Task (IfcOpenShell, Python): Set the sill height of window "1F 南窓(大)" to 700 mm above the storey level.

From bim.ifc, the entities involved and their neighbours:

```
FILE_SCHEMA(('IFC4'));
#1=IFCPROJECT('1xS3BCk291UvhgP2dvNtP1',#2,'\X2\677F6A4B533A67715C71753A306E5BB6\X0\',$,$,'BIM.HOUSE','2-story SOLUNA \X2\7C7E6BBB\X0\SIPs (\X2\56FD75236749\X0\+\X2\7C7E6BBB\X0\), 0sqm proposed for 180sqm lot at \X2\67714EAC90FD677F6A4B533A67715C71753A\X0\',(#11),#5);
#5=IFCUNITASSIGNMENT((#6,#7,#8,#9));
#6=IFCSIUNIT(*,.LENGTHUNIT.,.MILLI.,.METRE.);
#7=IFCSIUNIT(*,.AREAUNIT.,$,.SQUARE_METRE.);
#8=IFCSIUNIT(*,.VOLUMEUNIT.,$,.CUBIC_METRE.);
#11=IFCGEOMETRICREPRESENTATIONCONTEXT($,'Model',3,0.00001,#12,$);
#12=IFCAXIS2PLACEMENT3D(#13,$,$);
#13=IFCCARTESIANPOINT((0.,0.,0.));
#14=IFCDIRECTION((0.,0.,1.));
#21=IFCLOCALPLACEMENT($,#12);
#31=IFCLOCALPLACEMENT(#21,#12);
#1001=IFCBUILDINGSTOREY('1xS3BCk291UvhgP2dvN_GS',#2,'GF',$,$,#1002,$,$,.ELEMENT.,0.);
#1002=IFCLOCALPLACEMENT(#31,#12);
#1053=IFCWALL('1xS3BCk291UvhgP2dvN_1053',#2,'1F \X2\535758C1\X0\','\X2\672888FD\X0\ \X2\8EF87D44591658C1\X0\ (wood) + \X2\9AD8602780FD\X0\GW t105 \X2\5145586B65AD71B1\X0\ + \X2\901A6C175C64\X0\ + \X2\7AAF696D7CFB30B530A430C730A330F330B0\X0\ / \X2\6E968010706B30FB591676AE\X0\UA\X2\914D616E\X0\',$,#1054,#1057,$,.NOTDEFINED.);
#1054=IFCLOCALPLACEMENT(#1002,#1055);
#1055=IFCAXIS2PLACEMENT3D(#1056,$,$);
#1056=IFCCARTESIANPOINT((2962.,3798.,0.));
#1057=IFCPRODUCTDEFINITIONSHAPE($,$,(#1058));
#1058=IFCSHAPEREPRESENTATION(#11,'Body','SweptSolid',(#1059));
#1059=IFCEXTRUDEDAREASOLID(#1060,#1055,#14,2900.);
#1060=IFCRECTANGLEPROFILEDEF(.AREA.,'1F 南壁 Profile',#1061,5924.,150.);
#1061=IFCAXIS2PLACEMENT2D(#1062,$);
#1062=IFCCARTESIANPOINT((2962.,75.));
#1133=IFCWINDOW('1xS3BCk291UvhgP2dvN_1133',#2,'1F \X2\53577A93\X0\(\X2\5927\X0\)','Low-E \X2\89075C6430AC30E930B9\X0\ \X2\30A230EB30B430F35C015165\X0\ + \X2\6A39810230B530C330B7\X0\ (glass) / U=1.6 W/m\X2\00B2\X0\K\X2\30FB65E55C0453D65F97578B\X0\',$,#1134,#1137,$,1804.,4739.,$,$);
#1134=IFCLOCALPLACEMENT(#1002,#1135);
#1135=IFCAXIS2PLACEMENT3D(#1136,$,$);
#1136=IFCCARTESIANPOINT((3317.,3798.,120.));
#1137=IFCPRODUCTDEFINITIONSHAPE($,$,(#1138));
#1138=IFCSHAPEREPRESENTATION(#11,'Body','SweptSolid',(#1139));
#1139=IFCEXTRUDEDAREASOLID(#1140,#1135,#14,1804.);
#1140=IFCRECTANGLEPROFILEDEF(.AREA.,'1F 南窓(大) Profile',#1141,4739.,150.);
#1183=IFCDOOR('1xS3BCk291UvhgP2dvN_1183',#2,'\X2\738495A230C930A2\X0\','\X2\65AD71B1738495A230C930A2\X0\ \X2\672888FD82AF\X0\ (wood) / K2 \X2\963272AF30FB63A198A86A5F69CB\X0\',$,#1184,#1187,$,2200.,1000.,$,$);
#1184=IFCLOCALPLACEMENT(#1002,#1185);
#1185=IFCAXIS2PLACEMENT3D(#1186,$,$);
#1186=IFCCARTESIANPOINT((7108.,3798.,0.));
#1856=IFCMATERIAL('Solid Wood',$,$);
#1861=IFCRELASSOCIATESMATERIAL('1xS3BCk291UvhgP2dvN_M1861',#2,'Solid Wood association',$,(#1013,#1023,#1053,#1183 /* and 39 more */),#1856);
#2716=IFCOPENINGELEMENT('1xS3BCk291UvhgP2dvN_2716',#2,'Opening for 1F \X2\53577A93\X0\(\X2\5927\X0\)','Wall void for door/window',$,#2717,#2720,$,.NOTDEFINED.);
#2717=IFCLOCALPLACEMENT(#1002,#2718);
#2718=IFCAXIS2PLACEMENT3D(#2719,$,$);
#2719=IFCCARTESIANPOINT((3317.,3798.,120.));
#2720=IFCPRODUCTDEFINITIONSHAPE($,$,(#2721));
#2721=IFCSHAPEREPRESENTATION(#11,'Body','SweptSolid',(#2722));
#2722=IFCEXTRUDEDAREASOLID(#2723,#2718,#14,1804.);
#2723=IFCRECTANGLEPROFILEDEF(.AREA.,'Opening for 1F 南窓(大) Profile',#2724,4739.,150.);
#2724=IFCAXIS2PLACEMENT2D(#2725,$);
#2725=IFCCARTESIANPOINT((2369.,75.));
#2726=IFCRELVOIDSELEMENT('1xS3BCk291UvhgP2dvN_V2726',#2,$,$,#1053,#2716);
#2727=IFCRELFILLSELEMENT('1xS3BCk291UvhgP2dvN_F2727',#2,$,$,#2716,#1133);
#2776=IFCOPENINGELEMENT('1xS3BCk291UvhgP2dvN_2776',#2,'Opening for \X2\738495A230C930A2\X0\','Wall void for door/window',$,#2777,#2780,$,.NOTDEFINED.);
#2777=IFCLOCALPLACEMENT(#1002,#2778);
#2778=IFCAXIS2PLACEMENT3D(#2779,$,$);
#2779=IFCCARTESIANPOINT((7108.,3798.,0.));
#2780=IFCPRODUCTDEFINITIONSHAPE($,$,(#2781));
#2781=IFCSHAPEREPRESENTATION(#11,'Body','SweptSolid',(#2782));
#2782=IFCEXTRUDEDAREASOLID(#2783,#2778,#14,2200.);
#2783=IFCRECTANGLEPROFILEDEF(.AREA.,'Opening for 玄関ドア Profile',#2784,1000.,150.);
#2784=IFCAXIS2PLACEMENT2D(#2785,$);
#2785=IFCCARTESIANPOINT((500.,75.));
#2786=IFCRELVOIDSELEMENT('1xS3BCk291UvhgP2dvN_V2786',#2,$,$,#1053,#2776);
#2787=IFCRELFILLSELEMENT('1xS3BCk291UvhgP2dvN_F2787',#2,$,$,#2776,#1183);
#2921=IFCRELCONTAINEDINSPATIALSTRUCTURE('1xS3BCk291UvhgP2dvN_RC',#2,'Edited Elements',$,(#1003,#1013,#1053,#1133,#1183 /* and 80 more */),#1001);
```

```python
import numpy as np
import ifcopenshell
import ifcopenshell.api.geometry
import ifcopenshell.geom
import ifcopenshell.util.element
import ifcopenshell.util.placement
import ifcopenshell.util.shape
import ifcopenshell.util.unit

model = ifcopenshell.open("bim.ifc")
unit_scale = ifcopenshell.util.unit.calculate_unit_scale(model)

window = model.by_guid("1xS3BCk291UvhgP2dvN_1133")
opening = window.FillsVoids[0].RelatingOpeningElement
storey = ifcopenshell.util.element.get_container(window, ifc_class="IfcBuildingStorey")
level = ifcopenshell.util.placement.get_local_placement(storey.ObjectPlacement)[2, 3]

# The opening's origin need not be at the sill, so measure its lowest point.
shape = ifcopenshell.geom.create_shape(ifcopenshell.geom.settings(), opening)
bottom = ifcopenshell.util.shape.get_shape_bottom_elevation(shape, shape.geometry) / unit_scale
dz = level + 0.7 / unit_scale - bottom

shift = np.array([0.0, 0.0, dz])
# The window is not placed relative to its opening, so move both.
for product in (opening, window):
    matrix = ifcopenshell.util.placement.get_local_placement(product.ObjectPlacement)
    matrix[:3, 3] += shift
    ifcopenshell.api.geometry.edit_object_placement(model, product=product, matrix=matrix, is_si=False)

print(f"moved by {dz * unit_scale:+.3f} m")

model.write("bim_rev.ifc")
```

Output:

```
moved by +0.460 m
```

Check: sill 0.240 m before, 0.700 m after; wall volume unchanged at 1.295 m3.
